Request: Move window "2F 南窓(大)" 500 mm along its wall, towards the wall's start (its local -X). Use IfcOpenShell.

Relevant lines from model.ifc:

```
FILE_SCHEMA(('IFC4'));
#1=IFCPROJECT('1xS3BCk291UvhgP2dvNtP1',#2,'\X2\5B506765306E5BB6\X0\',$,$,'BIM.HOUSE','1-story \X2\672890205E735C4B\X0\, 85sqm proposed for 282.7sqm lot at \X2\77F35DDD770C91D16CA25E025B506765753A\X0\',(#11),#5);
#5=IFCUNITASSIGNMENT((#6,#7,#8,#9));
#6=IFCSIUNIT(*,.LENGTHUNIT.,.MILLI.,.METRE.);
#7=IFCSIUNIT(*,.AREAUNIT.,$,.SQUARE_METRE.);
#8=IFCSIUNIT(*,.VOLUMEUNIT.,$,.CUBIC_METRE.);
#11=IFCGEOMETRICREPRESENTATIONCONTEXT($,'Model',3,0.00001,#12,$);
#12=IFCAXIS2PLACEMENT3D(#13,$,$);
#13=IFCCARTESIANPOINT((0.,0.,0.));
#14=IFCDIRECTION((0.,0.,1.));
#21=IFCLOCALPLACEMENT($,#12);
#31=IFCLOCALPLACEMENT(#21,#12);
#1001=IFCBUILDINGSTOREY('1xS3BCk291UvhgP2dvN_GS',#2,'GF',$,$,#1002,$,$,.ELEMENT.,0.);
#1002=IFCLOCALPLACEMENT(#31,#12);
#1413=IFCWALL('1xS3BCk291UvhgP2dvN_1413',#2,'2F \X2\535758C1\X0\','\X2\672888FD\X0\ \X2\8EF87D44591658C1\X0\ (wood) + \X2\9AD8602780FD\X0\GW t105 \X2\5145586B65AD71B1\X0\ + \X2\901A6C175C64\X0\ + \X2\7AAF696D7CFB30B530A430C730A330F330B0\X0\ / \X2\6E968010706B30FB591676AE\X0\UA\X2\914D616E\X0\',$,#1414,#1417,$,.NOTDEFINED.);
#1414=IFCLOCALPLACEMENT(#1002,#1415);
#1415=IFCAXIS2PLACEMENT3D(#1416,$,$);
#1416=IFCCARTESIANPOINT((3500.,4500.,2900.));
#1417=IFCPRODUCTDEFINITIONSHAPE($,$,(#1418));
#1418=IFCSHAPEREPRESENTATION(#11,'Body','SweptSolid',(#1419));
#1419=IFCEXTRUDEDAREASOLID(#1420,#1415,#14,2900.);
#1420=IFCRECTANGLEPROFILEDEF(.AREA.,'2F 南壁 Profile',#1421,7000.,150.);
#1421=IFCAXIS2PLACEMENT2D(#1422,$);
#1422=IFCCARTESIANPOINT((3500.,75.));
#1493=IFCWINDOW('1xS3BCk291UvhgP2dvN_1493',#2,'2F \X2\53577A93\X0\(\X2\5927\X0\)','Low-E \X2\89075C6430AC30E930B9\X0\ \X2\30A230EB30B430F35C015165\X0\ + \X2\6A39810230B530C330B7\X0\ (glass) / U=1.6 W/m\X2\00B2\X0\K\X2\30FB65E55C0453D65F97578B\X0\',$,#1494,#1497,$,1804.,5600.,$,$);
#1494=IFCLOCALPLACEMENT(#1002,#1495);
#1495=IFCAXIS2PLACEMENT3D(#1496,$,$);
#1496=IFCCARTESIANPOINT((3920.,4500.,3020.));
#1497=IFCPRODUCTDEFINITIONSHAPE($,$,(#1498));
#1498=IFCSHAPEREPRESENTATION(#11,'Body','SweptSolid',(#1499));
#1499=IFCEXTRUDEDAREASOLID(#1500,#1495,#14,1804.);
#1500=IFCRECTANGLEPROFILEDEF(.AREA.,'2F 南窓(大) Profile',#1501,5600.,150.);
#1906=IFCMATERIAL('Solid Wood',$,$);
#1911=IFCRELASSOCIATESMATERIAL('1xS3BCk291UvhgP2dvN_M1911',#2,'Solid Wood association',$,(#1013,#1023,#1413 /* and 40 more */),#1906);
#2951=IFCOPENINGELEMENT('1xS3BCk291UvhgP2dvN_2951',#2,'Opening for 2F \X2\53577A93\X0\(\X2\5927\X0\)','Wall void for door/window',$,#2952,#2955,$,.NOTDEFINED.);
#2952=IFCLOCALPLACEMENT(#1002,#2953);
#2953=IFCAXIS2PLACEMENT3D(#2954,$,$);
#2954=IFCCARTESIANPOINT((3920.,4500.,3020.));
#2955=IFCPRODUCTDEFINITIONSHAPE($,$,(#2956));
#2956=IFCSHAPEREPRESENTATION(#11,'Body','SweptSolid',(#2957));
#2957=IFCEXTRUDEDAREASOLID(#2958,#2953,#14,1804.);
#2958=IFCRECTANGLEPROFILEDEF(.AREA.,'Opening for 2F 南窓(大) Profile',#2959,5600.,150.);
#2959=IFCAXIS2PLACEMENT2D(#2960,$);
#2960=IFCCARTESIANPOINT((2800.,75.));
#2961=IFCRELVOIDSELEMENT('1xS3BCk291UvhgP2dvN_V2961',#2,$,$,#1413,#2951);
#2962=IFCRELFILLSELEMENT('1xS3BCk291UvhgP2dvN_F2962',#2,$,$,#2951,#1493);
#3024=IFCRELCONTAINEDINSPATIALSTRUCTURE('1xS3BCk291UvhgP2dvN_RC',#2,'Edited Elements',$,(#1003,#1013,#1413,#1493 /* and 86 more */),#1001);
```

```python
import ifcopenshell
import ifcopenshell.api.geometry
import ifcopenshell.util.placement

model = ifcopenshell.open("model.ifc")

window = model.by_guid("1xS3BCk291UvhgP2dvN_1493")
opening = window.FillsVoids[0].RelatingOpeningElement
wall = opening.VoidsElements[0].RelatingBuildingElement

wall_matrix = ifcopenshell.util.placement.get_local_placement(wall.ObjectPlacement)
shift = wall_matrix[:3, 0] * -500.0
before = ifcopenshell.util.placement.get_local_placement(window.ObjectPlacement)[:3, 3].copy()

# The window is not placed relative to its opening, so move both.
for product in (opening, window):
    matrix = ifcopenshell.util.placement.get_local_placement(product.ObjectPlacement)
    matrix[:3, 3] += shift
    ifcopenshell.api.geometry.edit_object_placement(model, product=product, matrix=matrix, is_si=False)

after = ifcopenshell.util.placement.get_local_placement(window.ObjectPlacement)[:3, 3]
print("window moved by", (after - before).round(3) + 0.0)

model.write("model_rev.ifc")
```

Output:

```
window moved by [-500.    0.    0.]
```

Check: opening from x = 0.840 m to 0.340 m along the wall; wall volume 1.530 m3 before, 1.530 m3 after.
